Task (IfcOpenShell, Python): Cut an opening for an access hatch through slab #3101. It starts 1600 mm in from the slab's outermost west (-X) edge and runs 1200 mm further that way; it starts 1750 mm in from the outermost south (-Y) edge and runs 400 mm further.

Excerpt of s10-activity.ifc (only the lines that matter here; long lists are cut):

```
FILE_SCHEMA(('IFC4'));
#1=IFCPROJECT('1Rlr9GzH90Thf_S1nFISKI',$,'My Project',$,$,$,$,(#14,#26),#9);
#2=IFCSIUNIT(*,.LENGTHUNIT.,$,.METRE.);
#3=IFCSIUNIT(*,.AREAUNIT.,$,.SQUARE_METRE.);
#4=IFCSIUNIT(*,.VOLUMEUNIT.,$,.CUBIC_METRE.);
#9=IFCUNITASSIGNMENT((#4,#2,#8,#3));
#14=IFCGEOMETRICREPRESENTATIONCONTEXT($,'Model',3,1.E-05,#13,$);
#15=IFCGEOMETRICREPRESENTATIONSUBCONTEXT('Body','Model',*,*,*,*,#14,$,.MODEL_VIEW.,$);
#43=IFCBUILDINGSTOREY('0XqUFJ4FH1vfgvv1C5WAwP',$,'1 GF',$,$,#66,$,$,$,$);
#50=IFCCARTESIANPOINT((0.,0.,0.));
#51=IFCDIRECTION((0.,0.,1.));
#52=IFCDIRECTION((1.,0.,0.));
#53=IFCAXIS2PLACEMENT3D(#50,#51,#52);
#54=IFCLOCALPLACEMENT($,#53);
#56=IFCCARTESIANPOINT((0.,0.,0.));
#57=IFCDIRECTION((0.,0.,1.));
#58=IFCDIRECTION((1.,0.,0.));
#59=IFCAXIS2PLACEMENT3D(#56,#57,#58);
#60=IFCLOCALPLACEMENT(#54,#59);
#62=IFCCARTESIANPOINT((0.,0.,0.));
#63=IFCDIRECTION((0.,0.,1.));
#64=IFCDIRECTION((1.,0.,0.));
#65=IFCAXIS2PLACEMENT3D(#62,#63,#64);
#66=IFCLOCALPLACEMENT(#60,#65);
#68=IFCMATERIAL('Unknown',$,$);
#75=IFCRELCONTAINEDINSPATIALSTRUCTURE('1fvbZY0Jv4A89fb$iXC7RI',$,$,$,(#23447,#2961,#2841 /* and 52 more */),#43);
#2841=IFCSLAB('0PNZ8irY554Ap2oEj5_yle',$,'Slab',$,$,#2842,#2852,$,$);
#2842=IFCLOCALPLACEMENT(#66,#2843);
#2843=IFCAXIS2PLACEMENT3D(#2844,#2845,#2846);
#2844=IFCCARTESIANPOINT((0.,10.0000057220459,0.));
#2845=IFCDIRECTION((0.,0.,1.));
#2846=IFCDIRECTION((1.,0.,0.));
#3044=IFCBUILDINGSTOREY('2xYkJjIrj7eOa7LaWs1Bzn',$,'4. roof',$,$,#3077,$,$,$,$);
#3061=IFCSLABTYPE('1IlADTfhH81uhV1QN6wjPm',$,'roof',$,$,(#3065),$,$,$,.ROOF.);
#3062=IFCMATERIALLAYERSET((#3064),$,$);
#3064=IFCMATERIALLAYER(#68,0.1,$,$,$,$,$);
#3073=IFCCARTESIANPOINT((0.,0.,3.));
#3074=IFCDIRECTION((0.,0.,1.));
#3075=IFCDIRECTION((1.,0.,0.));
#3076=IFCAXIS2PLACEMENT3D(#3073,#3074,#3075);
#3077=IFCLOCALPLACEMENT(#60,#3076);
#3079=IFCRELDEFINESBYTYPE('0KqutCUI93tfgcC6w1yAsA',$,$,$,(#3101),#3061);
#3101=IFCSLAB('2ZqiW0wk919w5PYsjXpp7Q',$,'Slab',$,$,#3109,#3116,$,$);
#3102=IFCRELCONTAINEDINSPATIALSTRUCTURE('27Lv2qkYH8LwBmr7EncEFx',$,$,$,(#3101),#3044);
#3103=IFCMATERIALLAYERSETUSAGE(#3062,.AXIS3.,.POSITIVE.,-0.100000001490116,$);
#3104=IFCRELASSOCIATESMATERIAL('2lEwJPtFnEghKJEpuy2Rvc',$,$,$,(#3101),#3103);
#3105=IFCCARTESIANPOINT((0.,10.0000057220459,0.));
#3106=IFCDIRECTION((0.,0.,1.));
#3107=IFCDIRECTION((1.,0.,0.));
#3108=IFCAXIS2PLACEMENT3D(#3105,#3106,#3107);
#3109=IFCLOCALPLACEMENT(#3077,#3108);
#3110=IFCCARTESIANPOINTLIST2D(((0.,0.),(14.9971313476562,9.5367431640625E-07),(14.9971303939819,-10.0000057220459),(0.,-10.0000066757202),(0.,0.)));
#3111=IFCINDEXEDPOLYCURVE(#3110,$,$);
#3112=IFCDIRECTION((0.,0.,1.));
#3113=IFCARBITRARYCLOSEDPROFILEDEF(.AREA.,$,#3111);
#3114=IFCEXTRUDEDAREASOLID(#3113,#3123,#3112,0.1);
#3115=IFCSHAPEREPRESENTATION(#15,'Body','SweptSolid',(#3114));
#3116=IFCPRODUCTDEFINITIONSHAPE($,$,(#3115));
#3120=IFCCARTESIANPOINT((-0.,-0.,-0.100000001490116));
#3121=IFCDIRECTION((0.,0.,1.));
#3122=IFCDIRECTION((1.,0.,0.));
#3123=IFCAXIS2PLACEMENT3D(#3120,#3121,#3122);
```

```python
import numpy as np
import ifcopenshell
import ifcopenshell.api.feature
import ifcopenshell.api.geometry
import ifcopenshell.api.root
import ifcopenshell.geom
import ifcopenshell.util.placement
import ifcopenshell.util.representation
import ifcopenshell.util.shape
import ifcopenshell.util.unit

model = ifcopenshell.open("s10-activity.ifc")
unit_scale = ifcopenshell.util.unit.calculate_unit_scale(model)
settings = ifcopenshell.geom.settings()


def volume(element):
    """Net volume in cubic metres, openings subtracted."""
    shape = ifcopenshell.geom.create_shape(settings, element)
    return ifcopenshell.util.shape.get_volume(shape.geometry)


slab = model.by_guid("2ZqiW0wk919w5PYsjXpp7Q")
before = volume(slab)

# Extent in the slab's own axes, in metres. The edges named are its -X and -Y sides.
slab_shape = ifcopenshell.geom.create_shape(settings, slab)
vertices = ifcopenshell.util.shape.get_vertices(slab_shape.geometry)
x_min, y_min, bottom = vertices.min(axis=0)
top = vertices[:, 2].max()

opening = ifcopenshell.api.root.create_entity(model, ifc_class="IfcOpeningElement", name="Access hatch opening", predefined_type="OPENING")
context = ifcopenshell.util.representation.get_context(model, "Model", "Body", "MODEL_VIEW")
width, depth = 1.2, 0.4
outline = [(0.0, 0.0), (width, 0.0), (width, depth), (0.0, depth), (0.0, 0.0)]
# Overshoot both faces by 50 mm so the cut is clean.
shape = ifcopenshell.api.geometry.add_slab_representation(
    model, context=context, depth=top - bottom + 0.1, polyline=outline
)
ifcopenshell.api.geometry.assign_representation(model, product=opening, representation=shape)

matrix = ifcopenshell.util.placement.get_local_placement(slab.ObjectPlacement)
matrix[:, 3] = matrix @ np.append(np.array([x_min + 1.6, y_min + 1.75, bottom - 0.05]) / unit_scale, 1.0)
ifcopenshell.api.geometry.edit_object_placement(model, product=opening, matrix=matrix, is_si=False)
ifcopenshell.api.feature.add_feature(model, feature=opening, element=slab)

after = volume(slab)

print(f"slab volume {before:.3f} -> {after:.3f} m3")

model.write("s10-activity-out.ifc")
```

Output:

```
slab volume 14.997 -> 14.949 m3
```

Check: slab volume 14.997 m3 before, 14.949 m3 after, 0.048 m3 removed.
